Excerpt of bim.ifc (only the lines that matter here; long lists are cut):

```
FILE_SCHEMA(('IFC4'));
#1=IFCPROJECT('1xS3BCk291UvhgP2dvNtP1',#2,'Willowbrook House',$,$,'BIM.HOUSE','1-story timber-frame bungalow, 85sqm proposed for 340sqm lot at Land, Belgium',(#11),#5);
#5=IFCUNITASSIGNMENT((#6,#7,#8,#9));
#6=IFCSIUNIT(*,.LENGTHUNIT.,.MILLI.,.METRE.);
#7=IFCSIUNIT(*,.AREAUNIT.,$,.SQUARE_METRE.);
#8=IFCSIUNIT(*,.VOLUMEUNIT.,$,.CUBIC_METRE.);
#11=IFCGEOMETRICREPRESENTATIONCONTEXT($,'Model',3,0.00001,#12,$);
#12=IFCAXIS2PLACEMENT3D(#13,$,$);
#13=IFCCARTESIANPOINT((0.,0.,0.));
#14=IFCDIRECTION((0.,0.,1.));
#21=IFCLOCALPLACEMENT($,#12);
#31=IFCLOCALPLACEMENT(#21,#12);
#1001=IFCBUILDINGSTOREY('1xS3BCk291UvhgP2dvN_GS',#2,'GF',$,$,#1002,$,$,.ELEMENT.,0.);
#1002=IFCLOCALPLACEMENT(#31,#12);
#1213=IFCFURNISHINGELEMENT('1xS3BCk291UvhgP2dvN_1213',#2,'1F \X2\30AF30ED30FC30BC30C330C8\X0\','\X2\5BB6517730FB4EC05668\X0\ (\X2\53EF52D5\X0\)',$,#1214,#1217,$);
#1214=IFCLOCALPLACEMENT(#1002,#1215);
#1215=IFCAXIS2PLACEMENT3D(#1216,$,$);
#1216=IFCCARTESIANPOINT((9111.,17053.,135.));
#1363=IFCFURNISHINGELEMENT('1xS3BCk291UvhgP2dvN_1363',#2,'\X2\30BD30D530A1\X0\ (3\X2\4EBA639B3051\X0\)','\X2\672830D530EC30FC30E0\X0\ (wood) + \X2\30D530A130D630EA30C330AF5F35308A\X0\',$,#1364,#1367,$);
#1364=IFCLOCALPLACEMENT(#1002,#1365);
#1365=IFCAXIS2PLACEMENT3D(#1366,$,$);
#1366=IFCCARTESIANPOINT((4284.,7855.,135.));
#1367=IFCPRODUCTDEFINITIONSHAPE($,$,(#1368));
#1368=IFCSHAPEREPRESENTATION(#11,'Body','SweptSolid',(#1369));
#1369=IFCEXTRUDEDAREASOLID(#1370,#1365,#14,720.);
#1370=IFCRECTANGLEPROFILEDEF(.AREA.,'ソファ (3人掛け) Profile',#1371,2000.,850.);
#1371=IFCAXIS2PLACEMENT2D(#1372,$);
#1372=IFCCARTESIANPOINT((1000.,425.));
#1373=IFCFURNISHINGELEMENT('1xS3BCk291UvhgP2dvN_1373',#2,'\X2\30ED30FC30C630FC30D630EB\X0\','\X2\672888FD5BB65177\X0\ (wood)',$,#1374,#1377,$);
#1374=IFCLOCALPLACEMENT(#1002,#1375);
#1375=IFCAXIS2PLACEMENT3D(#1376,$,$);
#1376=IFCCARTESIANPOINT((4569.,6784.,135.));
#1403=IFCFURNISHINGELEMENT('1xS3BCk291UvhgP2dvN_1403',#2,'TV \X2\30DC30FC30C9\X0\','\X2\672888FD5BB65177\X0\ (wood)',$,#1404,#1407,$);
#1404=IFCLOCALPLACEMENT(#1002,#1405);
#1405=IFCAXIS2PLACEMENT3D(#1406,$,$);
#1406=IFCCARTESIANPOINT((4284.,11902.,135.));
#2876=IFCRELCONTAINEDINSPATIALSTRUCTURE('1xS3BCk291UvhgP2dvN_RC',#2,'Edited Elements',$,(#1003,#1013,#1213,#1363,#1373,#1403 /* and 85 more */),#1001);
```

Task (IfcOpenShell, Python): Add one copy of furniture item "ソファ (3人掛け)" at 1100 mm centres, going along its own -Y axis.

```python
import ifcopenshell
import ifcopenshell.api.geometry
import ifcopenshell.api.root
import ifcopenshell.util.element
import ifcopenshell.util.placement
import ifcopenshell.util.unit

model = ifcopenshell.open("bim.ifc")
unit_scale = ifcopenshell.util.unit.calculate_unit_scale(model)


def reuse_history(source, copy):
    """copy_class also copies each property set's owner history, people and application; keep the originals."""
    for rel in copy.IsDefinedBy:
        if rel.is_a("IfcRelDefinesByProperties") and (history := rel.RelatingPropertyDefinition.OwnerHistory):
            rel.RelatingPropertyDefinition.OwnerHistory = source.OwnerHistory
            ifcopenshell.util.element.remove_deep2(model, history)


source = model.by_guid("1xS3BCk291UvhgP2dvN_1363")
base = ifcopenshell.util.placement.get_local_placement(source.ObjectPlacement)
step = -base[:3, 1] * 1.1 / unit_scale

for i in range(1, 2):
    copy = ifcopenshell.api.root.copy_class(model, product=source)
    copy.Representation = ifcopenshell.util.element.copy_deep(
        model, source.Representation, exclude=["IfcGeometricRepresentationContext", "IfcRepresentationMap"]
    )
    reuse_history(source, copy)
    matrix = base.copy()
    matrix[:3, 3] += i * step
    print("added at", matrix[:3, 3].round(3) + 0.0)
    ifcopenshell.api.geometry.edit_object_placement(model, product=copy, matrix=matrix, is_si=False)

model.write("bim-out.ifc")
```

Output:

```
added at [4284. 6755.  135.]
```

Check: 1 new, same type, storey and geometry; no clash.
